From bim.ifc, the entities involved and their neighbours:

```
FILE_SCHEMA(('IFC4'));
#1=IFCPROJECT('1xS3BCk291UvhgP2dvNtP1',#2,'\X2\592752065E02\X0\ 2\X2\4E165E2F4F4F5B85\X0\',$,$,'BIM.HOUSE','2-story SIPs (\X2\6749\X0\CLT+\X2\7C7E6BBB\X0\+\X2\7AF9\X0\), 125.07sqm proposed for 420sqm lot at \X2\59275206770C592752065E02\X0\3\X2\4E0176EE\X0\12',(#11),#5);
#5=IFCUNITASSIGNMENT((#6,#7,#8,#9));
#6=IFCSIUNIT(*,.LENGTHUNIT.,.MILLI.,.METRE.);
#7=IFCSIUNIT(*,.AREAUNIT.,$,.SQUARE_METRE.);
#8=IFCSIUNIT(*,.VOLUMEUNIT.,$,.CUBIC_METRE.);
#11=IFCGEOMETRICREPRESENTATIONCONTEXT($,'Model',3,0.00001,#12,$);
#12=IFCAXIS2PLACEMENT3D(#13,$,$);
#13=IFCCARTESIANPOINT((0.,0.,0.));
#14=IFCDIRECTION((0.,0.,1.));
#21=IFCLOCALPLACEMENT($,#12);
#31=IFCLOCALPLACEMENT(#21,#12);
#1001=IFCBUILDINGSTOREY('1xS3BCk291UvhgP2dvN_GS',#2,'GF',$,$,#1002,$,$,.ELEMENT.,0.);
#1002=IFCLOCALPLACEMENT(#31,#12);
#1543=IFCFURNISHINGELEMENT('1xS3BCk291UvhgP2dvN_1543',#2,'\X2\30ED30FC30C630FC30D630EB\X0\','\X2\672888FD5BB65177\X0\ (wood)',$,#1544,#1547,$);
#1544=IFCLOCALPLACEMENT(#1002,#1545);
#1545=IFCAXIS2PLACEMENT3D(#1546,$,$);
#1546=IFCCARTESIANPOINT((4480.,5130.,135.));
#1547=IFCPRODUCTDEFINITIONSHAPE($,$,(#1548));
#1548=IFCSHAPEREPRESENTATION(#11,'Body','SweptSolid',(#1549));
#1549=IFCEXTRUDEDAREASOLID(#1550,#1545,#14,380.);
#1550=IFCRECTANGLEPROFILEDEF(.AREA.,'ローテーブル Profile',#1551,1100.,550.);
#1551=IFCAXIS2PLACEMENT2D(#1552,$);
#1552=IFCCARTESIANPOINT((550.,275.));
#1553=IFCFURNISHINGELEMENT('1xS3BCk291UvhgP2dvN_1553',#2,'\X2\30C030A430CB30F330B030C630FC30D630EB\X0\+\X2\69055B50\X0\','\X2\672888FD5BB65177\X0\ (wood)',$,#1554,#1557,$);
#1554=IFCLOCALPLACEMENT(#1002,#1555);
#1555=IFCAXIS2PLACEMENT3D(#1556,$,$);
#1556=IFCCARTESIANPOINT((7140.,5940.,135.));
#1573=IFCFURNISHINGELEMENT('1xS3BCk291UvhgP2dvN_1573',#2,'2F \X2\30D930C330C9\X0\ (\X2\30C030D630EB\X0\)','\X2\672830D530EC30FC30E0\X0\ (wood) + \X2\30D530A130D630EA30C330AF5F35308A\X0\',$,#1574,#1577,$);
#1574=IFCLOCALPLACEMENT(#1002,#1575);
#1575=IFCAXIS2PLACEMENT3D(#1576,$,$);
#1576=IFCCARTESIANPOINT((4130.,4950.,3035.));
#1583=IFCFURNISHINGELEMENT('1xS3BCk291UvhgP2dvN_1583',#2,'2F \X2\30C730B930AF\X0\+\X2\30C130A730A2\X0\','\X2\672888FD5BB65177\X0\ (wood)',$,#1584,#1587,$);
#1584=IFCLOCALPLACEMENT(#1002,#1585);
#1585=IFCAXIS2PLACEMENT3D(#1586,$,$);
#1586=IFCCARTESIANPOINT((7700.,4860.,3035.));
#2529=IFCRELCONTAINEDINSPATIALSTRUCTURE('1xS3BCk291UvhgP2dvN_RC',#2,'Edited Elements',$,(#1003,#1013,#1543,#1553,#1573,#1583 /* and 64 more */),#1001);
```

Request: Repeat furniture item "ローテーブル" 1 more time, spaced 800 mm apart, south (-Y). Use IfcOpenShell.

```python
import numpy as np
import ifcopenshell
import ifcopenshell.api.geometry
import ifcopenshell.api.root
import ifcopenshell.util.element
import ifcopenshell.util.placement
import ifcopenshell.util.unit

model = ifcopenshell.open("bim.ifc")
unit_scale = ifcopenshell.util.unit.calculate_unit_scale(model)


def reuse_history(source, copy):
    """copy_class also copies each property set's owner history, people and application; keep the originals."""
    for rel in copy.IsDefinedBy:
        if rel.is_a("IfcRelDefinesByProperties") and (history := rel.RelatingPropertyDefinition.OwnerHistory):
            rel.RelatingPropertyDefinition.OwnerHistory = source.OwnerHistory
            ifcopenshell.util.element.remove_deep2(model, history)


source = model.by_id(1543)
base = ifcopenshell.util.placement.get_local_placement(source.ObjectPlacement)
step = np.array([0.0, -1.0, 0.0]) * 0.8 / unit_scale

for i in range(1, 2):
    copy = ifcopenshell.api.root.copy_class(model, product=source)
    copy.Representation = ifcopenshell.util.element.copy_deep(
        model, source.Representation, exclude=["IfcGeometricRepresentationContext", "IfcRepresentationMap"]
    )
    reuse_history(source, copy)
    matrix = base.copy()
    matrix[:3, 3] += i * step
    print("added at", matrix[:3, 3].round(3) + 0.0)
    ifcopenshell.api.geometry.edit_object_placement(model, product=copy, matrix=matrix, is_si=False)

model.write("bim_edited.ifc")
```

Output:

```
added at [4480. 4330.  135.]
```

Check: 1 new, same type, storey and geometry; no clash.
